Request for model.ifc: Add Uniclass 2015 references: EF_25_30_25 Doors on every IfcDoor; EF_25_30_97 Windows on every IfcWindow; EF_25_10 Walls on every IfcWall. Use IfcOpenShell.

First a look at what the model holds.

```python
import ifcopenshell

model = ifcopenshell.open("model.ifc")
print(model.schema)
print("classifications:", [c.Name for c in model.by_type("IfcClassification")])
for ifc_class in ("IfcDoor", "IfcRoof", "IfcStair", "IfcWall", "IfcWindow"):
    print(ifc_class, len(model.by_type(ifc_class)))
```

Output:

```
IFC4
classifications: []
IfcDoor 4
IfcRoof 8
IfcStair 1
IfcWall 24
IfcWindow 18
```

```python
import ifcopenshell
import ifcopenshell.api.classification

model = ifcopenshell.open("model.ifc")

system = ifcopenshell.api.classification.add_classification(model, classification="Uniclass 2015")

codes = {
    "IfcDoor": ("EF_25_30_25", "Doors"),
    "IfcWindow": ("EF_25_30_97", "Windows"),
    "IfcWall": ("EF_25_10", "Walls"),
}
for ifc_class, (code, name) in codes.items():
    products = model.by_type(ifc_class)
    ifcopenshell.api.classification.add_reference(
        model, products=products, classification=system, identification=code, name=name
    )
    print(code, len(products))

model.write("model_rev.ifc")
```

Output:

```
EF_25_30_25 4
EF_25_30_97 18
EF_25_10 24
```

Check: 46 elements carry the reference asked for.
